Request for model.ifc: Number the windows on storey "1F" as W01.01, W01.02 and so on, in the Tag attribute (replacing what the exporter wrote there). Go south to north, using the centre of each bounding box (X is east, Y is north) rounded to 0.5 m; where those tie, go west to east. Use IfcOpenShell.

First a look at what the model holds.

```python
import ifcopenshell
import ifcopenshell.util.element
import ifcopenshell.util.placement

model = ifcopenshell.open("model.ifc")
print(model.schema)
storey = next(s for s in model.by_type("IfcBuildingStorey") if s.Name == "1F")
windows = [e for e in ifcopenshell.util.element.get_decomposition(storey) if e.is_a("IfcWindow")]
for e in sorted(windows, key=lambda e: e.id()):
    origin = ifcopenshell.util.placement.get_local_placement(e.ObjectPlacement)[:3, 3]
    print(e.id(), e.Tag, e.Name, origin.round(2) + 0.0, sep=" | ")
```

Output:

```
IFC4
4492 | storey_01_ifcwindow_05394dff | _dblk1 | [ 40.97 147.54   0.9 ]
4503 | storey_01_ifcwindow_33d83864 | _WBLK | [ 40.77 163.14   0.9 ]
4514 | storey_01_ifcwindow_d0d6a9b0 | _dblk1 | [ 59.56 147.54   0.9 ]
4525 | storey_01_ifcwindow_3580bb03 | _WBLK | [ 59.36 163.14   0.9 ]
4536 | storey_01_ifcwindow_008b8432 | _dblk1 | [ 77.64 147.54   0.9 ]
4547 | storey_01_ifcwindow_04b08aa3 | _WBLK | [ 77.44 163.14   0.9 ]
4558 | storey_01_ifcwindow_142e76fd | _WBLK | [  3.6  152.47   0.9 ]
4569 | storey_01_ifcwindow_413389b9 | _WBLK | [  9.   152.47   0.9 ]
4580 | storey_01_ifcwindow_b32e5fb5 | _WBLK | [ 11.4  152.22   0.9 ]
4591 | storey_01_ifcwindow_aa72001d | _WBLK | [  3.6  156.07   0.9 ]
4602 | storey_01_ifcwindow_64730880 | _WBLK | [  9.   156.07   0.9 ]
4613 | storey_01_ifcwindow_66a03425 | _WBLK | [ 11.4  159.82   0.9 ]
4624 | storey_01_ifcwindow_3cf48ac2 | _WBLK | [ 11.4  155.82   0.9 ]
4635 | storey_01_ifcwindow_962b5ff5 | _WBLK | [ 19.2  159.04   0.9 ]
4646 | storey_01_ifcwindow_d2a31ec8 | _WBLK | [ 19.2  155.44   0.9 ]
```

```python
import ifcopenshell
import ifcopenshell.geom
import ifcopenshell.util.element
import ifcopenshell.util.shape

model = ifcopenshell.open("model.ifc")
settings = ifcopenshell.geom.settings()
settings.set("use-world-coords", True)


def centre(element):
    shape = ifcopenshell.geom.create_shape(settings, element)
    return ifcopenshell.util.shape.get_bbox_centroid(shape.geometry)


storey = next(s for s in model.by_type("IfcBuildingStorey") if s.Name == "1F")
windows = [e for e in ifcopenshell.util.element.get_decomposition(storey) if e.is_a("IfcWindow")]

# Insertion points can sit at a corner or the storey origin, so sort by the geometry (in metres).
centres = {e: centre(e) for e in windows}
windows.sort(key=lambda e: (round(centres[e][1] / 0.5), centres[e][0]))

for i, e in enumerate(windows, start=1):
    number = f"W01.{i:02d}"
    e.Tag = number
    print(e.id(), number)

model.write("model_rev.ifc")
```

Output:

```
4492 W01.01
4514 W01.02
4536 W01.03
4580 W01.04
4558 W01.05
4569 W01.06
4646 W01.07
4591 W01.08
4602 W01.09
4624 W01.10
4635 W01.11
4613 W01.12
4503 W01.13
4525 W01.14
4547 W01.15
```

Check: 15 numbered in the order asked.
